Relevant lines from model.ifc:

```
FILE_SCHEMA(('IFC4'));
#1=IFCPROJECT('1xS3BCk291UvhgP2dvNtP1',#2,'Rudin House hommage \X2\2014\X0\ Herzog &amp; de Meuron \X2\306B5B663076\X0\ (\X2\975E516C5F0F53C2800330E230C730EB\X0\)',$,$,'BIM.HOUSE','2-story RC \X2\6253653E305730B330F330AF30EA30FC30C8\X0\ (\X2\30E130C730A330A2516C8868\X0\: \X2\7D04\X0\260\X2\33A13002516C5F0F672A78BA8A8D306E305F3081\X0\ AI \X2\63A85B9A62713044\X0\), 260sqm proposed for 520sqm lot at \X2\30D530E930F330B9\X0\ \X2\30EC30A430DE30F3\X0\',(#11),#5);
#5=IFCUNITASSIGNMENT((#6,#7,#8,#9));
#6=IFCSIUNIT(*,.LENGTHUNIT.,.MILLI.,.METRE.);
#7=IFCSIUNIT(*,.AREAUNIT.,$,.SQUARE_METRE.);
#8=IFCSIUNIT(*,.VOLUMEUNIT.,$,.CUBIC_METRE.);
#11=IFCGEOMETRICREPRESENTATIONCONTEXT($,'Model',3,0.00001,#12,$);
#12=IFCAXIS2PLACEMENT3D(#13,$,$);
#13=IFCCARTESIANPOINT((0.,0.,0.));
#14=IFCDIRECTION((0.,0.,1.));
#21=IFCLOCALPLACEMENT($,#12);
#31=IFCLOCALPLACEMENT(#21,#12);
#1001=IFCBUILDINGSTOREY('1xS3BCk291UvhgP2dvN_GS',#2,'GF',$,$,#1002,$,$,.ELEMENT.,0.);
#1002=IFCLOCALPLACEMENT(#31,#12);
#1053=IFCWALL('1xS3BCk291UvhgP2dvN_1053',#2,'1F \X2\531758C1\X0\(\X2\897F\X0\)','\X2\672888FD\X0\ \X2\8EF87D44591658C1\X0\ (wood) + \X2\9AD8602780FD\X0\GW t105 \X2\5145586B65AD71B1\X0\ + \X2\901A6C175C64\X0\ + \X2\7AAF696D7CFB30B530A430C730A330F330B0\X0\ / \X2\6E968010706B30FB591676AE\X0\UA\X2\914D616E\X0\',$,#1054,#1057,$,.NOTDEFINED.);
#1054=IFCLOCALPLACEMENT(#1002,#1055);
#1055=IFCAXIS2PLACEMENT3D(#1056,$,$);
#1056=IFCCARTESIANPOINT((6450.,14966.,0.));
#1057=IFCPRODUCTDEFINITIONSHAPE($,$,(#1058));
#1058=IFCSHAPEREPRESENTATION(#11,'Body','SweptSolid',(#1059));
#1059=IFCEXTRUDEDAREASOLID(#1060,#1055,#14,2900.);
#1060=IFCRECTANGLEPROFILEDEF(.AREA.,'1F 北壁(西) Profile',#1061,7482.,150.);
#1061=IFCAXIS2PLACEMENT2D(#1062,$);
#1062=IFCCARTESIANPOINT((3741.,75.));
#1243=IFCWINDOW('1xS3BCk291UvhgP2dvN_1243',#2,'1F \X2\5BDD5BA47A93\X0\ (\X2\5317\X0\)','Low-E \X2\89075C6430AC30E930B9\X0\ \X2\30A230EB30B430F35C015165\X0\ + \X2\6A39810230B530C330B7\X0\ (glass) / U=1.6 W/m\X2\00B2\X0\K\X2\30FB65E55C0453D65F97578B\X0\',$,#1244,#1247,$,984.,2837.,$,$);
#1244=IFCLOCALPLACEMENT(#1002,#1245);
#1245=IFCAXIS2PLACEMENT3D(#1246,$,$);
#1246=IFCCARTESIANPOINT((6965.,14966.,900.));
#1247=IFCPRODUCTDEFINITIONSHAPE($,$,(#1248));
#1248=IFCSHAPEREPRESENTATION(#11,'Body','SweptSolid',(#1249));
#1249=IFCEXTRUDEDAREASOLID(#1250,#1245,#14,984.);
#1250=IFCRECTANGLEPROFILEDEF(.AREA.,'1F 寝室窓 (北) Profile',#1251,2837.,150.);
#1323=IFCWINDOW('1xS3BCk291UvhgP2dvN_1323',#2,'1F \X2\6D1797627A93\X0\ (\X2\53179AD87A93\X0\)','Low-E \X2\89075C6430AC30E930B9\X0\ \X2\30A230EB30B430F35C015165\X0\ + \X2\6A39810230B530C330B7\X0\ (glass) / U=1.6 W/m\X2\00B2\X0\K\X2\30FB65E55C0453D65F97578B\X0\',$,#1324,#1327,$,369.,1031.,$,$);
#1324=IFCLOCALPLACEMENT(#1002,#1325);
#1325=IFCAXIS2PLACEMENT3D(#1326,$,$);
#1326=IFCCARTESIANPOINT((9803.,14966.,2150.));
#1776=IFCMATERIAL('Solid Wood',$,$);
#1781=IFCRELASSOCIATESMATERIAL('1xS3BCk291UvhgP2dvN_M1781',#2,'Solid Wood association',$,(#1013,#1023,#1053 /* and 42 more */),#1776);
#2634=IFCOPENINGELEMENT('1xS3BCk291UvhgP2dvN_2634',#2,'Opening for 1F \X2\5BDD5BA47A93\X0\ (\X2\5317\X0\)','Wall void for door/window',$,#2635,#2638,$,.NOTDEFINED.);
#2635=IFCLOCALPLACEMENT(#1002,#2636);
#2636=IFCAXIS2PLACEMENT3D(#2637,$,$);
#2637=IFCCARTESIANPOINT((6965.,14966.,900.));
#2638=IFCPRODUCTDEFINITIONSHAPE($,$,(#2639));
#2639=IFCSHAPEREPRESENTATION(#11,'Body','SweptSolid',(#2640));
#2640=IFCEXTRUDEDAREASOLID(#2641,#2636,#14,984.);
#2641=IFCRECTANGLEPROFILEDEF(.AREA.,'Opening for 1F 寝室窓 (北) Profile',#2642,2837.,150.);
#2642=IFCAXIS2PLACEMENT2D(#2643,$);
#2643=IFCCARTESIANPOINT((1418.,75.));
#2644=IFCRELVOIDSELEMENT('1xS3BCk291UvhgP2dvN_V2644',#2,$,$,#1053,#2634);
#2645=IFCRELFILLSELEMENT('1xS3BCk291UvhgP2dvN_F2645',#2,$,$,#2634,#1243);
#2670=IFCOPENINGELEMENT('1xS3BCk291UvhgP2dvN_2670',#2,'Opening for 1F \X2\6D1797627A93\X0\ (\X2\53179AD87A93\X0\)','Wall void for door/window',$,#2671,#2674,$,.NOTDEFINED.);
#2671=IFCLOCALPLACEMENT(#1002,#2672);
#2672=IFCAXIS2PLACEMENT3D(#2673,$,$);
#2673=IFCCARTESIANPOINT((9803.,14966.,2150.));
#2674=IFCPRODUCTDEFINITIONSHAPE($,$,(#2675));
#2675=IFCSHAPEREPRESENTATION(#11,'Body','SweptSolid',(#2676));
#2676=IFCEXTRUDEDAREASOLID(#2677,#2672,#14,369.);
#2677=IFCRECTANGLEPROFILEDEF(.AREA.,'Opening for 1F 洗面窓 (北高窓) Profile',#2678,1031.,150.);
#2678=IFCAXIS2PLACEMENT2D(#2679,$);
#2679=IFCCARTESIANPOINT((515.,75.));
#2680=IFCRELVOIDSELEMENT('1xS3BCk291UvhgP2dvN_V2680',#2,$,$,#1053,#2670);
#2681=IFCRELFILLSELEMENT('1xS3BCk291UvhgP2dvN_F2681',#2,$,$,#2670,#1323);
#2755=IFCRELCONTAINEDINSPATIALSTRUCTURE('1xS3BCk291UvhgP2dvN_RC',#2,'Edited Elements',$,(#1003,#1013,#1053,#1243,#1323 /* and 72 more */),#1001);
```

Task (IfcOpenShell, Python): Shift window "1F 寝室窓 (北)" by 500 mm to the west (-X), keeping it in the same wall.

```python
import ifcopenshell
import ifcopenshell.api.geometry
import ifcopenshell.util.placement
import ifcopenshell.util.unit

model = ifcopenshell.open("model.ifc")
unit_scale = ifcopenshell.util.unit.calculate_unit_scale(model)

window = model.by_id(1243)
opening = window.FillsVoids[0].RelatingOpeningElement
wall = opening.VoidsElements[0].RelatingBuildingElement

wall_matrix = ifcopenshell.util.placement.get_local_placement(wall.ObjectPlacement)
shift = wall_matrix[:3, 0] * -0.5 / unit_scale
before = ifcopenshell.util.placement.get_local_placement(window.ObjectPlacement)[:3, 3].copy()

# The window is not placed relative to its opening, so move both.
for product in (opening, window):
    matrix = ifcopenshell.util.placement.get_local_placement(product.ObjectPlacement)
    matrix[:3, 3] += shift
    ifcopenshell.api.geometry.edit_object_placement(model, product=product, matrix=matrix, is_si=False)

after = ifcopenshell.util.placement.get_local_placement(window.ObjectPlacement)[:3, 3]
print("window moved by", (after - before).round(3) + 0.0)

model.write("model_v2.ifc")
```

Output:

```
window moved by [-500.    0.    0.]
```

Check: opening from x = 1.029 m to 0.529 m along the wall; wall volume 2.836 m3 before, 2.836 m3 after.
